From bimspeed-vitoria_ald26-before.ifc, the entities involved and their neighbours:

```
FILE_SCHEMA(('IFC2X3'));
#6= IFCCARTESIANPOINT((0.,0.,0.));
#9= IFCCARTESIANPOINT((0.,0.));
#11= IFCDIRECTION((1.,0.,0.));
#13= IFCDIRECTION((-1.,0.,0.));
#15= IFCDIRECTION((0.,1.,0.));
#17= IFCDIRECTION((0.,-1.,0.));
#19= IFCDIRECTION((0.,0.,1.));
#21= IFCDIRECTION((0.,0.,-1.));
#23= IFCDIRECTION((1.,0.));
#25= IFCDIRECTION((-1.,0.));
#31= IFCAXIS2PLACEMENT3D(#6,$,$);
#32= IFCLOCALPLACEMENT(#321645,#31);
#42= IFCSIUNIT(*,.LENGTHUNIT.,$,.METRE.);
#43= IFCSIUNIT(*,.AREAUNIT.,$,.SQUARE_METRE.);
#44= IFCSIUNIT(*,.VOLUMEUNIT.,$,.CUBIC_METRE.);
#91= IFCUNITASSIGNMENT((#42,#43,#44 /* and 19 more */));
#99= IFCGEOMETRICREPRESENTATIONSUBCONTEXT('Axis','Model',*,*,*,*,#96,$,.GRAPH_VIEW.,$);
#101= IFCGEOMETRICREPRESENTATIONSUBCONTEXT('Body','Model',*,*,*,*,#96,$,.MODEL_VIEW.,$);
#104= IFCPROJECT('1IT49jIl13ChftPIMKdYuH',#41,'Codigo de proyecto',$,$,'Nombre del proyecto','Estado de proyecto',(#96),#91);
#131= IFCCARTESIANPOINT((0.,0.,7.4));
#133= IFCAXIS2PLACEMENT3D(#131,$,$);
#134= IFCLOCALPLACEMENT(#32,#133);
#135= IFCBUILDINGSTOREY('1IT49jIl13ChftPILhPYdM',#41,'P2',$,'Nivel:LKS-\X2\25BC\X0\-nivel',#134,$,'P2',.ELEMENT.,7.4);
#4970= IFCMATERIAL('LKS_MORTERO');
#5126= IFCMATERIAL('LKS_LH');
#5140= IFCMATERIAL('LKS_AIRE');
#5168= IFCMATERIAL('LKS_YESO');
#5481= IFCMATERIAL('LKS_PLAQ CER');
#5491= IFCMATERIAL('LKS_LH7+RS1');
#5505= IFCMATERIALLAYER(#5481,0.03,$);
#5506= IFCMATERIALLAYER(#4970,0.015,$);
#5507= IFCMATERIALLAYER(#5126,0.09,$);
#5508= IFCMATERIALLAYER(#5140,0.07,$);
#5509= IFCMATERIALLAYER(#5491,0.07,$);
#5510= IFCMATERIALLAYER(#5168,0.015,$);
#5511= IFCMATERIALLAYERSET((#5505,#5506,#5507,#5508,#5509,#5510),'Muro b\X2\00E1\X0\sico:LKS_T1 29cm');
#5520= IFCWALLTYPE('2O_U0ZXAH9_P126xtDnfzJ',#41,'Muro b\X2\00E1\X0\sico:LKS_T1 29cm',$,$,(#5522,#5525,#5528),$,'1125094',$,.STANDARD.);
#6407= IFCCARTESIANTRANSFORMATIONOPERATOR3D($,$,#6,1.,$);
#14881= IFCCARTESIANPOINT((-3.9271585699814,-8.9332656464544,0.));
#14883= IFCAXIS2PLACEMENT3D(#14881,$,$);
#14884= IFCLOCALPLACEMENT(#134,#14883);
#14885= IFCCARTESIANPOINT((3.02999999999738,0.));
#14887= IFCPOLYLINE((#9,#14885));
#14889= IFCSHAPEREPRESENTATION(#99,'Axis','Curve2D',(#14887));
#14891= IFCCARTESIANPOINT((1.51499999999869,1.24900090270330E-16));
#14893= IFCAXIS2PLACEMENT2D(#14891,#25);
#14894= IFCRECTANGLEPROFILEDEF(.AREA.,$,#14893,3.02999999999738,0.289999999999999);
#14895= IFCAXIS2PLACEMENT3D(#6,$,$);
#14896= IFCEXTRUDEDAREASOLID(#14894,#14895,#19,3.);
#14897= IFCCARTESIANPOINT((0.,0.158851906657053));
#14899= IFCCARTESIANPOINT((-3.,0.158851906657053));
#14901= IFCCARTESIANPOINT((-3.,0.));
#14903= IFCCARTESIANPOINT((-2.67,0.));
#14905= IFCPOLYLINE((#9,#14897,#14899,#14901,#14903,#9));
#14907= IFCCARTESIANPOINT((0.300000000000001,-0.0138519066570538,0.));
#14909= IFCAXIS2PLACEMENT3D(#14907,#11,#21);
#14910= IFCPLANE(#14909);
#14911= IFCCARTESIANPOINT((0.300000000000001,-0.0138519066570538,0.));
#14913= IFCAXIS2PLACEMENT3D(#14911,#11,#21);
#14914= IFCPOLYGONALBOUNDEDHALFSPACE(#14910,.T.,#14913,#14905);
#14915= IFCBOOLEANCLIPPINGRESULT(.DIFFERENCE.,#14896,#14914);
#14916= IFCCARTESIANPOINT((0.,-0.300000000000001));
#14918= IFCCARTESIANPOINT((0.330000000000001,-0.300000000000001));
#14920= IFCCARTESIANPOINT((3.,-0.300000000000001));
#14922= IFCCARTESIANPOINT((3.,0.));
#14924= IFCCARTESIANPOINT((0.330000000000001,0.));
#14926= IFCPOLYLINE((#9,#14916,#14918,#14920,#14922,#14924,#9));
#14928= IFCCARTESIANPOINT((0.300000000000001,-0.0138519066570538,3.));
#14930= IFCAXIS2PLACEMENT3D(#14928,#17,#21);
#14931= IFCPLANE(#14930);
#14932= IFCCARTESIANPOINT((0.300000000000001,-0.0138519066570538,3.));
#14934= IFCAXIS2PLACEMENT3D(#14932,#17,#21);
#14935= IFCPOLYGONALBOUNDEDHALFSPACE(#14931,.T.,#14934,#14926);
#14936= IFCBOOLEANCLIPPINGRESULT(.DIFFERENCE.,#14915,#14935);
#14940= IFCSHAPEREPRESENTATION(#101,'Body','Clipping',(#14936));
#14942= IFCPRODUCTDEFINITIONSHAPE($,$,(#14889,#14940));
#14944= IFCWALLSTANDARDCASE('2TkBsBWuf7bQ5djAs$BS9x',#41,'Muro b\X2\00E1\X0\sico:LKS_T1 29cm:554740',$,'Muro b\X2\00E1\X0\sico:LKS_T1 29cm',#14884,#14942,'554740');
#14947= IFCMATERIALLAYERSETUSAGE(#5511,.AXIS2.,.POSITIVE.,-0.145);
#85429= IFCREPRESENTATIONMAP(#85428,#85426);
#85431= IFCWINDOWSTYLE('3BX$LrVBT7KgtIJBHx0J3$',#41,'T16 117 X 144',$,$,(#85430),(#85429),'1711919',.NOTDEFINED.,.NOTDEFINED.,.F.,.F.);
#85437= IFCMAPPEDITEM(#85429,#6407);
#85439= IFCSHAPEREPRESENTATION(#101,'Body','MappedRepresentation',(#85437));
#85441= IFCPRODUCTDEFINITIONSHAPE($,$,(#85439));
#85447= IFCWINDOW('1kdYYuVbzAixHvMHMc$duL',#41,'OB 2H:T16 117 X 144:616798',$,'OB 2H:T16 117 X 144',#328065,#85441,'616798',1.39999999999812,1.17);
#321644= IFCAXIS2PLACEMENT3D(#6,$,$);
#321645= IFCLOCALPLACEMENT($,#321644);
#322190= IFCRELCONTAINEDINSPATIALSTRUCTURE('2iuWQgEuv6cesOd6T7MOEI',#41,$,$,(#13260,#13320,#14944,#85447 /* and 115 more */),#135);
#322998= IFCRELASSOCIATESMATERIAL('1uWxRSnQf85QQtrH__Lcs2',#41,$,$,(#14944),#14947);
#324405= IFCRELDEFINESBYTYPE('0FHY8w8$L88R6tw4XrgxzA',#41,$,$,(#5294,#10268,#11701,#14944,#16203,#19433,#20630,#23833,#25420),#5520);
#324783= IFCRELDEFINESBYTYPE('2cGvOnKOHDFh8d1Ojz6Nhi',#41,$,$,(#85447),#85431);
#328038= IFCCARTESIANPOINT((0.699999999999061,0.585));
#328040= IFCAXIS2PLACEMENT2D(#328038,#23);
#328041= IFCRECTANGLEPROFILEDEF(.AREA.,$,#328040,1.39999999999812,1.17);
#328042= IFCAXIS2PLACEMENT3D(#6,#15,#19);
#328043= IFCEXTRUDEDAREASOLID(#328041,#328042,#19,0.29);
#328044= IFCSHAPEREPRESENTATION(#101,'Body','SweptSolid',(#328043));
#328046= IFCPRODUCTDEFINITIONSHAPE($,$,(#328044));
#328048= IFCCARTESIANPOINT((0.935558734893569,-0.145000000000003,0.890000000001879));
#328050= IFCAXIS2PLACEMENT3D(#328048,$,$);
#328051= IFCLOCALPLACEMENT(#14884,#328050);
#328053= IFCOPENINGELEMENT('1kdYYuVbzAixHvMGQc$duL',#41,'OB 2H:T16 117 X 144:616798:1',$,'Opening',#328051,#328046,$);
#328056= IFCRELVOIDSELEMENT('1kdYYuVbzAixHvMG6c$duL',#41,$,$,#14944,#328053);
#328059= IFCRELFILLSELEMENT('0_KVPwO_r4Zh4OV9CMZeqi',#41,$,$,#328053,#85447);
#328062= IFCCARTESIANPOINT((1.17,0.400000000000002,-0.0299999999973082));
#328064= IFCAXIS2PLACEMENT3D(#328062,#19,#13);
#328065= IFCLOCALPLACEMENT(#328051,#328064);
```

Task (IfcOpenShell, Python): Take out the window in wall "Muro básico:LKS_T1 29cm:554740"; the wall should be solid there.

```python
import ifcopenshell
import ifcopenshell.api.feature
import ifcopenshell.api.root
import ifcopenshell.geom
import ifcopenshell.util.shape

model = ifcopenshell.open("bimspeed-vitoria_ald26-before.ifc")
settings = ifcopenshell.geom.settings()


def volume(element):
    """Net volume in cubic metres, openings subtracted."""
    shape = ifcopenshell.geom.create_shape(settings, element)
    return ifcopenshell.util.shape.get_volume(shape.geometry)


window = model.by_guid("1kdYYuVbzAixHvMHMc$duL")
opening = window.FillsVoids[0].RelatingOpeningElement
wall = opening.VoidsElements[0].RelatingBuildingElement
before = volume(wall)

ifcopenshell.api.root.remove_product(model, product=window)
ifcopenshell.api.feature.remove_feature(model, feature=opening)

after = volume(wall)

print(f"wall volume {before:.3f} -> {after:.3f} m3")

model.write("bimspeed-vitoria_ald26-before_edited.ifc")
```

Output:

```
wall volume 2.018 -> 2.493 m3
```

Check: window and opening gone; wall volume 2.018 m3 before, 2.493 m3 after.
